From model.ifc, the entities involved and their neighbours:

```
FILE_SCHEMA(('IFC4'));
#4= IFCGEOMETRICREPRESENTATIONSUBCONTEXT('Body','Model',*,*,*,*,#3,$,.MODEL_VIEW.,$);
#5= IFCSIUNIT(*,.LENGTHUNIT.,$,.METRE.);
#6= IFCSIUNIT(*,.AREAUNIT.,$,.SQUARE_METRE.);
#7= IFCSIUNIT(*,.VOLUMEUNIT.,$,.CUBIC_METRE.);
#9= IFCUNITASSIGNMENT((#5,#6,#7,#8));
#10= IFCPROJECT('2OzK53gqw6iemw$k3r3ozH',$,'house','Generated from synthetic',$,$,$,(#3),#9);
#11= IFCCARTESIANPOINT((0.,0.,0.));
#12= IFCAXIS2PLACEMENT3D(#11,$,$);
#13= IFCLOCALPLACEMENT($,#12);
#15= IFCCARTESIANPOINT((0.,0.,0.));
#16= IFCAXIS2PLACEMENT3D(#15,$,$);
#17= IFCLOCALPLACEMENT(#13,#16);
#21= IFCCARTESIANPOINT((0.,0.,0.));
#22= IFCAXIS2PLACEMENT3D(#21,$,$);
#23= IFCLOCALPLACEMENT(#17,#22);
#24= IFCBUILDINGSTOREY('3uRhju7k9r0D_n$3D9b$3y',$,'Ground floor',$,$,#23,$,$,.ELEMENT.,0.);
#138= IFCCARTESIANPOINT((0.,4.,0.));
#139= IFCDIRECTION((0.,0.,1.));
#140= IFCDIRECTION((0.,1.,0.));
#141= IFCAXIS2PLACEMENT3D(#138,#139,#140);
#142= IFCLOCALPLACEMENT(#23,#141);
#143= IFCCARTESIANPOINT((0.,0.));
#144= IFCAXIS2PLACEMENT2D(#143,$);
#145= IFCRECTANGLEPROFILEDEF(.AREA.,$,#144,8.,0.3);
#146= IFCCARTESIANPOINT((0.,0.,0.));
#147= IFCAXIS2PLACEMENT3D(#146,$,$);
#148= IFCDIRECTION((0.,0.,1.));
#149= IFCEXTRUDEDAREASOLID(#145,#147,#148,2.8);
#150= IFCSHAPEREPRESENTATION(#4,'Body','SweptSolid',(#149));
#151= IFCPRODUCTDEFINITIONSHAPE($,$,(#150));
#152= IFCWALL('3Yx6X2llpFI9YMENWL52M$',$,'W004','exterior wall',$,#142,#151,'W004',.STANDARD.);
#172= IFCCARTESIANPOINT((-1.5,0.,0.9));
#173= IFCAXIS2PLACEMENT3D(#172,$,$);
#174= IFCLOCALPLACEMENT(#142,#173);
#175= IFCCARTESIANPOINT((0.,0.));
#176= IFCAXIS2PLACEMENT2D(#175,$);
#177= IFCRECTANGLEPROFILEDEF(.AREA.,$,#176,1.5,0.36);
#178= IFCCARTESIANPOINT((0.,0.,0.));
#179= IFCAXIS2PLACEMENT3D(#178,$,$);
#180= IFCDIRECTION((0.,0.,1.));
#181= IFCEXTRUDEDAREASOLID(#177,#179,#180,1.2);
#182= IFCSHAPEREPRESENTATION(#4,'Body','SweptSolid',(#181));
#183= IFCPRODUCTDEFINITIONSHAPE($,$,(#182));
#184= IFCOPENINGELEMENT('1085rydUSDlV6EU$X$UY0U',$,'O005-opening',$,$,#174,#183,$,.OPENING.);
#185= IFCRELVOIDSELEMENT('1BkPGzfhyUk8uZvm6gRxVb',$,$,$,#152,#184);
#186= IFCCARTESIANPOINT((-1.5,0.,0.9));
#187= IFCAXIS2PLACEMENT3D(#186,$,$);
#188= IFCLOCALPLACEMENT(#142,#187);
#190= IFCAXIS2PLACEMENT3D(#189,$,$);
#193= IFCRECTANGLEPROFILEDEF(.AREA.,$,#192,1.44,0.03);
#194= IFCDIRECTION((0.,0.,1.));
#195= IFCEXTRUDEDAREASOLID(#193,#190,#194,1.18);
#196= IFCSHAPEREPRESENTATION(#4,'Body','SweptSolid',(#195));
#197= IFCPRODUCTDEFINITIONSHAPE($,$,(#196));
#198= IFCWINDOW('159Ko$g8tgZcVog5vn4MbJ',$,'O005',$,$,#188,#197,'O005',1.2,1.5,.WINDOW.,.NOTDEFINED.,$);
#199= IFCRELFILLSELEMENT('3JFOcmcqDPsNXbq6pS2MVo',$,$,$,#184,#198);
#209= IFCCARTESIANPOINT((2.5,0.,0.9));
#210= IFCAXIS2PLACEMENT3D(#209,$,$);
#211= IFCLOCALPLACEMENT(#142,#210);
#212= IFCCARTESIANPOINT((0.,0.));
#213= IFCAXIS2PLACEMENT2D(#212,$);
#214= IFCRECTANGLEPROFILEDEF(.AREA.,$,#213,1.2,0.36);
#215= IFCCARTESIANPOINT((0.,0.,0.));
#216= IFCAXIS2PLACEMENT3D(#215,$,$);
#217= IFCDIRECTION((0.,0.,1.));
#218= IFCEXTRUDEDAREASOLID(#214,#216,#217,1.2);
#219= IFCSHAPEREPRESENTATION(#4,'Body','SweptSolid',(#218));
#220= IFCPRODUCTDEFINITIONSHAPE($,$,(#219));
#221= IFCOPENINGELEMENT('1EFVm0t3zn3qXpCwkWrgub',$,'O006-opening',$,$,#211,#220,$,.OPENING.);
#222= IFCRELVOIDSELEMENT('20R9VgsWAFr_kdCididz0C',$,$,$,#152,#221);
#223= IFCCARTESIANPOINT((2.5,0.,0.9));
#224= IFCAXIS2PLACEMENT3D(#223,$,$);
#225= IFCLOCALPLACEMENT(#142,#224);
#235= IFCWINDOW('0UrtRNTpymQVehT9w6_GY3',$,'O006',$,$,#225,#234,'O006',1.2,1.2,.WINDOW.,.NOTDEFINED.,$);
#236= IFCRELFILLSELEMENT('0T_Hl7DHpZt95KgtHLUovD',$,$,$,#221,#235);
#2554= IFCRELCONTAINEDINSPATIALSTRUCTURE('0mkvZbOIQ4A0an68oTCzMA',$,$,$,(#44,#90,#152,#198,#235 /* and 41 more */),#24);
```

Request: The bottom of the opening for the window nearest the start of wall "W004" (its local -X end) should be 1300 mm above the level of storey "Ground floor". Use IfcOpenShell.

```python
import numpy as np
import ifcopenshell
import ifcopenshell.api.geometry
import ifcopenshell.geom
import ifcopenshell.util.element
import ifcopenshell.util.placement
import ifcopenshell.util.shape
import ifcopenshell.util.unit

model = ifcopenshell.open("model.ifc")
unit_scale = ifcopenshell.util.unit.calculate_unit_scale(model)

window = model.by_guid("159Ko$g8tgZcVog5vn4MbJ")
opening = window.FillsVoids[0].RelatingOpeningElement
storey = ifcopenshell.util.element.get_container(window, ifc_class="IfcBuildingStorey")
level = ifcopenshell.util.placement.get_local_placement(storey.ObjectPlacement)[2, 3]

# The opening's origin need not be at the sill, so measure its lowest point.
shape = ifcopenshell.geom.create_shape(ifcopenshell.geom.settings(), opening)
bottom = ifcopenshell.util.shape.get_shape_bottom_elevation(shape, shape.geometry) / unit_scale
dz = level + 1.3 - bottom

shift = np.array([0.0, 0.0, dz])
# The window is not placed relative to its opening, so move both.
for product in (opening, window):
    matrix = ifcopenshell.util.placement.get_local_placement(product.ObjectPlacement)
    matrix[:3, 3] += shift
    ifcopenshell.api.geometry.edit_object_placement(model, product=product, matrix=matrix, is_si=False)

print(f"moved by {dz * unit_scale:+.3f} m")

model.write("model-out.ifc")
```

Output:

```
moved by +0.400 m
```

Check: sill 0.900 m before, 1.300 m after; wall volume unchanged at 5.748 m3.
